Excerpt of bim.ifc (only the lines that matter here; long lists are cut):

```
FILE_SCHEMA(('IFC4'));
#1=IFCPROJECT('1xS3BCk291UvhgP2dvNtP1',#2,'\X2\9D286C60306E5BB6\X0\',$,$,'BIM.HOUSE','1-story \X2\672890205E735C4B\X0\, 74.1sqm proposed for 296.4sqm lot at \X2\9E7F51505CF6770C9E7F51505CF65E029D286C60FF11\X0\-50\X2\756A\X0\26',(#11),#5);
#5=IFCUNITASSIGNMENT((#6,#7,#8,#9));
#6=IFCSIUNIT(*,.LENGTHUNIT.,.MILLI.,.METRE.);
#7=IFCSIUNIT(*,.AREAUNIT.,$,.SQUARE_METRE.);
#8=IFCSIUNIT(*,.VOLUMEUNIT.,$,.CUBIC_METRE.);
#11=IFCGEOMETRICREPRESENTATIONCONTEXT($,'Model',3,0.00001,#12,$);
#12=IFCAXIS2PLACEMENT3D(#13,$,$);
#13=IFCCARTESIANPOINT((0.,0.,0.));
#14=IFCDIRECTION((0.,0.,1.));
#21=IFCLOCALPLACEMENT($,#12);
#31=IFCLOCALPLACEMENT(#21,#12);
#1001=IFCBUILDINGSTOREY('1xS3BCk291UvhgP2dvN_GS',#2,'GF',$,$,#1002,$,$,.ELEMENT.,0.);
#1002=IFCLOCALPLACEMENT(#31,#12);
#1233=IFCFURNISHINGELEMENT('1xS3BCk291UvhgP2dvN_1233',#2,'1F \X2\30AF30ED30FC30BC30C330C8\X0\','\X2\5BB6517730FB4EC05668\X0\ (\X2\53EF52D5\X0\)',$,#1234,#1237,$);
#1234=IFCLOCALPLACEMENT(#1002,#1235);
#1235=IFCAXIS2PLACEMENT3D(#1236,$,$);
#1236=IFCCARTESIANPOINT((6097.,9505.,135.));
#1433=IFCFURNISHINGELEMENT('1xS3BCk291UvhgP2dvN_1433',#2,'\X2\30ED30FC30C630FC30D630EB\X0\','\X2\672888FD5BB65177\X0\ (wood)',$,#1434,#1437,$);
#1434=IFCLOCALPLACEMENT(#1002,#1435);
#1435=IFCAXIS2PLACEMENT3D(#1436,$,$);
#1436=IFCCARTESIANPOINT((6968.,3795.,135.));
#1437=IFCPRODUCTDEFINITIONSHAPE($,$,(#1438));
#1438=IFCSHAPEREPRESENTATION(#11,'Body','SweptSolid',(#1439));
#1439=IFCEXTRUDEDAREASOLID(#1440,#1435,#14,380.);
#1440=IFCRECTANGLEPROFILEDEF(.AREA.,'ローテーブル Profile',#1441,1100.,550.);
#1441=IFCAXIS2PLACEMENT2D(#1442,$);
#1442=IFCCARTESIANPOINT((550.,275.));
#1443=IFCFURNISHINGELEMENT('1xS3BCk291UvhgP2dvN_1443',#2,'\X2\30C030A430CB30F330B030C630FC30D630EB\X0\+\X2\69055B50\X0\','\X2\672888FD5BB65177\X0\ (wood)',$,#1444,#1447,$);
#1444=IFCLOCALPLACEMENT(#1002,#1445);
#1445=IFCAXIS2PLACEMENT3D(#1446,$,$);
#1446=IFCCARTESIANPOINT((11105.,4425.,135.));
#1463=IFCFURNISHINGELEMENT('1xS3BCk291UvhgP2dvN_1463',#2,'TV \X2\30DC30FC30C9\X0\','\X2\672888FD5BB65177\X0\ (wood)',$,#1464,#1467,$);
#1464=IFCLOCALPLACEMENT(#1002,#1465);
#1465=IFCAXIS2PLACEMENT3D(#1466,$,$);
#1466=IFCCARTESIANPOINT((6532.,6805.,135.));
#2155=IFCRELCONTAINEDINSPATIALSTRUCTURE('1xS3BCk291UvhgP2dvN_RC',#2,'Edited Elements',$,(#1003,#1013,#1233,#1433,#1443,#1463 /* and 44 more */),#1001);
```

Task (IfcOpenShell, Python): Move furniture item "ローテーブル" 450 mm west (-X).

```python
import ifcopenshell
import ifcopenshell.api.geometry
import ifcopenshell.util.placement
import ifcopenshell.util.unit

model = ifcopenshell.open("bim.ifc")
unit_scale = ifcopenshell.util.unit.calculate_unit_scale(model)

item = model.by_id(1433)
matrix = ifcopenshell.util.placement.get_local_placement(item.ObjectPlacement)
matrix[0, 3] -= 0.45 / unit_scale
ifcopenshell.api.geometry.edit_object_placement(model, product=item, matrix=matrix, is_si=False)

print(ifcopenshell.util.placement.get_local_placement(item.ObjectPlacement).round(3) + 0.0)

model.write("bim_v2.ifc")
```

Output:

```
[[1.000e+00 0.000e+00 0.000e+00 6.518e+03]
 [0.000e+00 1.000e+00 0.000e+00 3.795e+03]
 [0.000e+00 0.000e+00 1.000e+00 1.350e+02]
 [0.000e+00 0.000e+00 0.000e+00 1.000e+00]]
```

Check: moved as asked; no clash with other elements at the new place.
